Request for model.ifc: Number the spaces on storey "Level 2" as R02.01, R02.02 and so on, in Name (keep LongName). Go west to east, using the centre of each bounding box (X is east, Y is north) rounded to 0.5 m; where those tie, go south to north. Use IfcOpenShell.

First a look at what the model holds.

```python
import ifcopenshell
import ifcopenshell.util.element
import ifcopenshell.util.placement

model = ifcopenshell.open("model.ifc")
print(model.schema)
storey = next(s for s in model.by_type("IfcBuildingStorey") if s.Name == "Level 2")
spaces = [e for e in ifcopenshell.util.element.get_decomposition(storey) if e.is_a("IfcSpace")]
for e in sorted(spaces, key=lambda e: e.id()):
    origin = ifcopenshell.util.placement.get_local_placement(e.ObjectPlacement)[:3, 3]
    print(e.id(), e.Name, e.LongName, origin.round(2) + 0.0, sep=" | ")
```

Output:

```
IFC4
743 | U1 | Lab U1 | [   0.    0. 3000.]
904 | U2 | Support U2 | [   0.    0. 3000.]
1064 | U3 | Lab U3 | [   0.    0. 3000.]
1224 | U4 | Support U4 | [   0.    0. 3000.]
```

```python
import ifcopenshell
import ifcopenshell.geom
import ifcopenshell.util.element
import ifcopenshell.util.shape

model = ifcopenshell.open("model.ifc")
settings = ifcopenshell.geom.settings()
settings.set("use-world-coords", True)


def centre(element):
    shape = ifcopenshell.geom.create_shape(settings, element)
    return ifcopenshell.util.shape.get_bbox_centroid(shape.geometry)


storey = next(s for s in model.by_type("IfcBuildingStorey") if s.Name == "Level 2")
spaces = [e for e in ifcopenshell.util.element.get_decomposition(storey) if e.is_a("IfcSpace")]

# Insertion points can sit at a corner or the storey origin, so sort by the geometry (in metres).
centres = {e: centre(e) for e in spaces}
spaces.sort(key=lambda e: (round(centres[e][0] / 0.5), centres[e][1]))

for i, e in enumerate(spaces, start=1):
    number = f"R02.{i:02d}"
    e.Name = number
    print(e.id(), number)

model.write("model_updated.ifc")
```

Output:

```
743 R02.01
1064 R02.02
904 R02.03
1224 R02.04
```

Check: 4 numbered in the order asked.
